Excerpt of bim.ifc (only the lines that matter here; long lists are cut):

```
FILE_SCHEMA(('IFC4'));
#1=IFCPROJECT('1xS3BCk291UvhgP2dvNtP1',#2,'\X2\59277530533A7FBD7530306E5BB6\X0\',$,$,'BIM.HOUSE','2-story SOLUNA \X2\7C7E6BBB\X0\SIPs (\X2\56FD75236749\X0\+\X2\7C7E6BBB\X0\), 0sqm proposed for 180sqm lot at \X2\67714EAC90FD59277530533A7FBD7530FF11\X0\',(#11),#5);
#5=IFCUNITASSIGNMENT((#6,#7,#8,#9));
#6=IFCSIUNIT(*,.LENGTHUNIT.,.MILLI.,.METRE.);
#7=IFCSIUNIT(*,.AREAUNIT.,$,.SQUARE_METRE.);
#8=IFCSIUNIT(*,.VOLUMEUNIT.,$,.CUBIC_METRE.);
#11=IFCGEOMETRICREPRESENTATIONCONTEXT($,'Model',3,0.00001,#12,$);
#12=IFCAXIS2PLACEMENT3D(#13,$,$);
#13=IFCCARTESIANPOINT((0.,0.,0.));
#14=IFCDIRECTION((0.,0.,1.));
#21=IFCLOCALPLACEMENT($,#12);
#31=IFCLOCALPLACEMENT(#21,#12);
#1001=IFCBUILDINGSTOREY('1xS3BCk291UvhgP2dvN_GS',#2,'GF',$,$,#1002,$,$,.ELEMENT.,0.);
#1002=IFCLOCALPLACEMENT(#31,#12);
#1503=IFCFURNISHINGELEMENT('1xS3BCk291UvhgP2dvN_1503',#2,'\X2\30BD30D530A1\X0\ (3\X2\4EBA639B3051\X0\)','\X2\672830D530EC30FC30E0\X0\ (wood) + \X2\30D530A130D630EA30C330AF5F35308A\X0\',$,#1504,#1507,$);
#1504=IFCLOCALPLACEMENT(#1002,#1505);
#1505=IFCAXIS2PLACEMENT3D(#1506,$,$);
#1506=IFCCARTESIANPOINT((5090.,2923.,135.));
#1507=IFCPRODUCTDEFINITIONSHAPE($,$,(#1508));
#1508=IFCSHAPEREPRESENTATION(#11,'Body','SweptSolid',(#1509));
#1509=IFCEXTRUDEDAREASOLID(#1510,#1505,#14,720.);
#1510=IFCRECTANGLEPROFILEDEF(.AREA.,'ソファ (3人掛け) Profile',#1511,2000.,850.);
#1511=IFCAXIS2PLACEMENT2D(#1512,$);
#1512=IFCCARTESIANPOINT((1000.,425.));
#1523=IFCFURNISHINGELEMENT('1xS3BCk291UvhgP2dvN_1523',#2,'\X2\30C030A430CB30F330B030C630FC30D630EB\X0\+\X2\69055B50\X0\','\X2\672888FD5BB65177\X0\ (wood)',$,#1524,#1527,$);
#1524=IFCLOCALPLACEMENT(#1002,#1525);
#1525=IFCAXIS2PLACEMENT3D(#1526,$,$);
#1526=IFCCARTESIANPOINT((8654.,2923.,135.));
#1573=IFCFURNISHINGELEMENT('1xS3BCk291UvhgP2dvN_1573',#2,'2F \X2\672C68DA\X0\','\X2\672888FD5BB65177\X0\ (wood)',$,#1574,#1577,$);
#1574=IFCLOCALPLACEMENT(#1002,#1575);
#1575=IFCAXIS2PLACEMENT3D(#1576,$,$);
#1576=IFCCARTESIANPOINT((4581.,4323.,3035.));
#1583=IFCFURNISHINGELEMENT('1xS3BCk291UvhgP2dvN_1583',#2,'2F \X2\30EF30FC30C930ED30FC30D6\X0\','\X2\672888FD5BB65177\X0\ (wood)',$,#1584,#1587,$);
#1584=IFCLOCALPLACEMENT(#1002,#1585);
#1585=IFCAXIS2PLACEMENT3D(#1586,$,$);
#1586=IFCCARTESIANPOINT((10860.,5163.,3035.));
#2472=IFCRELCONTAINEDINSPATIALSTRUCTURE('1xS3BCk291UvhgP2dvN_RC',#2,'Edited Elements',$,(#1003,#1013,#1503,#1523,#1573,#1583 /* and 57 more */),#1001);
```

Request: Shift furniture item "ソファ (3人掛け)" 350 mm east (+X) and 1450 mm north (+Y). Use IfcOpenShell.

```python
import ifcopenshell
import ifcopenshell.api.geometry
import ifcopenshell.util.placement
import ifcopenshell.util.unit

model = ifcopenshell.open("bim.ifc")
unit_scale = ifcopenshell.util.unit.calculate_unit_scale(model)

item = model.by_id(1503)
matrix = ifcopenshell.util.placement.get_local_placement(item.ObjectPlacement)
matrix[0, 3] += 0.35 / unit_scale
matrix[1, 3] += 1.45 / unit_scale
ifcopenshell.api.geometry.edit_object_placement(model, product=item, matrix=matrix, is_si=False)

print(ifcopenshell.util.placement.get_local_placement(item.ObjectPlacement).round(3) + 0.0)

model.write("bim_v2.ifc")
```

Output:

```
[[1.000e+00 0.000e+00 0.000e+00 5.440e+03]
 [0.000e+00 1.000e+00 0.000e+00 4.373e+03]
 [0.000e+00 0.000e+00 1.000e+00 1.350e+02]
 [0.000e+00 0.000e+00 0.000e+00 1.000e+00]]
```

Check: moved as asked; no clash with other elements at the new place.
